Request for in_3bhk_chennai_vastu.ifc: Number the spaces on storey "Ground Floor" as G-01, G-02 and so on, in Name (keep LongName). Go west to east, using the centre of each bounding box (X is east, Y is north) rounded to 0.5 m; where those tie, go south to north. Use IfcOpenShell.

First a look at what the model holds.

```python
import ifcopenshell
import ifcopenshell.util.element
import ifcopenshell.util.placement

model = ifcopenshell.open("in_3bhk_chennai_vastu.ifc")
print(model.schema)
storey = next(s for s in model.by_type("IfcBuildingStorey") if s.Name == "Ground Floor")
spaces = [e for e in ifcopenshell.util.element.get_decomposition(storey) if e.is_a("IfcSpace")]
for e in sorted(spaces, key=lambda e: e.id()):
    origin = ifcopenshell.util.placement.get_local_placement(e.ObjectPlacement)[:3, 3]
    print(e.id(), e.Name, e.LongName, origin.round(2) + 0.0, sep=" | ")
```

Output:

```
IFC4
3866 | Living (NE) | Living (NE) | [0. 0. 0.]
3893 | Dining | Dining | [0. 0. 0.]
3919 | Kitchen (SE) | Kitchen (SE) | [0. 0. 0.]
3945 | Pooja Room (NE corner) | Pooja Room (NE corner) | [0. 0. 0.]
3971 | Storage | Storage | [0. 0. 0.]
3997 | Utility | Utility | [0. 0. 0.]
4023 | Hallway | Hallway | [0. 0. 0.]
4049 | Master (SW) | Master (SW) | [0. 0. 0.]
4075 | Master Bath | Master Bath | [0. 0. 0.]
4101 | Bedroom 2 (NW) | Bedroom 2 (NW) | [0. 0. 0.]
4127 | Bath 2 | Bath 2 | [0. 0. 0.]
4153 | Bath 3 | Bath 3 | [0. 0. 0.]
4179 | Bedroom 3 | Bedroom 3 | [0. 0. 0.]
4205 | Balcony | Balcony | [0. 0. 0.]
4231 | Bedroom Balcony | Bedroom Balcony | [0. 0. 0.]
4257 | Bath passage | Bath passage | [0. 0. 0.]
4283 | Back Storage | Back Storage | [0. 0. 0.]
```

```python
import ifcopenshell
import ifcopenshell.geom
import ifcopenshell.util.element
import ifcopenshell.util.shape

model = ifcopenshell.open("in_3bhk_chennai_vastu.ifc")
settings = ifcopenshell.geom.settings()
settings.set("use-world-coords", True)


def centre(element):
    shape = ifcopenshell.geom.create_shape(settings, element)
    return ifcopenshell.util.shape.get_bbox_centroid(shape.geometry)


storey = next(s for s in model.by_type("IfcBuildingStorey") if s.Name == "Ground Floor")
spaces = [e for e in ifcopenshell.util.element.get_decomposition(storey) if e.is_a("IfcSpace")]

# Insertion points can sit at a corner or the storey origin, so sort by the geometry (in metres).
centres = {e: centre(e) for e in spaces}
spaces.sort(key=lambda e: (round(centres[e][0] / 0.5), centres[e][1]))

for i, e in enumerate(spaces, start=1):
    number = f"G-{i:02d}"
    e.Name = number
    print(e.id(), number)

model.write("in_3bhk_chennai_vastu_rev.ifc")
```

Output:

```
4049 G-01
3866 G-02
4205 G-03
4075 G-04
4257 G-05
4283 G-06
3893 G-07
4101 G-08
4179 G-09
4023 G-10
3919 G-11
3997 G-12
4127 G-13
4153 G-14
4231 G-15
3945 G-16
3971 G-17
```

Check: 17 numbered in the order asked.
